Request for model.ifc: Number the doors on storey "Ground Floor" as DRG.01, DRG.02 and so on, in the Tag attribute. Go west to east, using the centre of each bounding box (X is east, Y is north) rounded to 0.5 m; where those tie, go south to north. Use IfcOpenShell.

First a look at what the model holds.

```python
import ifcopenshell
import ifcopenshell.util.element
import ifcopenshell.util.placement

model = ifcopenshell.open("model.ifc")
print(model.schema)
storey = next(s for s in model.by_type("IfcBuildingStorey") if s.Name == "Ground Floor")
doors = [e for e in ifcopenshell.util.element.get_decomposition(storey) if e.is_a("IfcDoor")]
for e in sorted(doors, key=lambda e: e.id()):
    origin = ifcopenshell.util.placement.get_local_placement(e.ObjectPlacement)[:3, 3]
    print(e.id(), e.Tag, e.Name, origin.round(2) + 0.0, sep=" | ")
```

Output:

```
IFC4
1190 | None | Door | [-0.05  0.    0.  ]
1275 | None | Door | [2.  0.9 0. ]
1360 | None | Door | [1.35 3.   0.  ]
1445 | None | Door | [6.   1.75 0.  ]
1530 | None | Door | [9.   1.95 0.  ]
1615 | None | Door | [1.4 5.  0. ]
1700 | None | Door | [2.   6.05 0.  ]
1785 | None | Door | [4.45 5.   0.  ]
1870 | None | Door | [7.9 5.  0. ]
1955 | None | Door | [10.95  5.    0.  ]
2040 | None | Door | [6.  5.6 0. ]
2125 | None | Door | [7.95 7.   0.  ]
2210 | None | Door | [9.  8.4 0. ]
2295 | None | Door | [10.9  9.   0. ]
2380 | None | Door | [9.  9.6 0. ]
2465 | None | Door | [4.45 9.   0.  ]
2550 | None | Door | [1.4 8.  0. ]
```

```python
import ifcopenshell
import ifcopenshell.geom
import ifcopenshell.util.element
import ifcopenshell.util.shape

model = ifcopenshell.open("model.ifc")
settings = ifcopenshell.geom.settings()
settings.set("use-world-coords", True)


def centre(element):
    shape = ifcopenshell.geom.create_shape(settings, element)
    return ifcopenshell.util.shape.get_bbox_centroid(shape.geometry)


storey = next(s for s in model.by_type("IfcBuildingStorey") if s.Name == "Ground Floor")
doors = [e for e in ifcopenshell.util.element.get_decomposition(storey) if e.is_a("IfcDoor")]

# Insertion points can sit at a corner or the storey origin, so sort by the geometry (in metres).
centres = {e: centre(e) for e in doors}
doors.sort(key=lambda e: (round(centres[e][0] / 0.5), centres[e][1]))

for i, e in enumerate(doors, start=1):
    number = f"DRG.{i:02d}"
    e.Tag = number
    print(e.id(), number)

model.write("model-out.ifc")
```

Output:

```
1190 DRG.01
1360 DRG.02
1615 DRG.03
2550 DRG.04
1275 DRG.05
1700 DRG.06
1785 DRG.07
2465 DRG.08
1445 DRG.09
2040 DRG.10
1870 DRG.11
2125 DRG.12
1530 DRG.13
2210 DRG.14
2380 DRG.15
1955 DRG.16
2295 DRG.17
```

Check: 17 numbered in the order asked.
